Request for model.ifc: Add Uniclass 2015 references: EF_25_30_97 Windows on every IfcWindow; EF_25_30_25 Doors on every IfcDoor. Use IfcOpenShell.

First a look at what the model holds.

```python
import ifcopenshell

model = ifcopenshell.open("model.ifc")
print(model.schema)
print("classifications:", [c.Name for c in model.by_type("IfcClassification")])
for ifc_class in ("IfcDoor", "IfcRoof", "IfcStair", "IfcWall", "IfcWindow"):
    print(ifc_class, len(model.by_type(ifc_class)))
```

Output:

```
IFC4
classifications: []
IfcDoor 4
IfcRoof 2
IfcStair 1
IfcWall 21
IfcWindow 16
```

```python
import ifcopenshell
import ifcopenshell.api.classification

model = ifcopenshell.open("model.ifc")

system = ifcopenshell.api.classification.add_classification(model, classification="Uniclass 2015")

codes = {
    "IfcWindow": ("EF_25_30_97", "Windows"),
    "IfcDoor": ("EF_25_30_25", "Doors"),
}
for ifc_class, (code, name) in codes.items():
    products = model.by_type(ifc_class)
    ifcopenshell.api.classification.add_reference(
        model, products=products, classification=system, identification=code, name=name
    )
    print(code, len(products))

model.write("model_updated.ifc")
```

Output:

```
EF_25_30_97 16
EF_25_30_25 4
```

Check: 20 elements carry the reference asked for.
